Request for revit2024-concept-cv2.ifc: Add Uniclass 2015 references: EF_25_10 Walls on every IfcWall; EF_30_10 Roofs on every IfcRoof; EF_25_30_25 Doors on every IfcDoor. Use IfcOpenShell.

First a look at what the model holds.

```python
import ifcopenshell

model = ifcopenshell.open("revit2024-concept-cv2.ifc")
print(model.schema)
print("classifications:", [c.Name for c in model.by_type("IfcClassification")])
for ifc_class in ("IfcDoor", "IfcRoof", "IfcStair", "IfcWall", "IfcWindow"):
    print(ifc_class, len(model.by_type(ifc_class)))
```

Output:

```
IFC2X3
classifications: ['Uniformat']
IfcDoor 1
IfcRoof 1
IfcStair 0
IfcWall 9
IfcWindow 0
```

```python
import ifcopenshell
import ifcopenshell.api.classification

model = ifcopenshell.open("revit2024-concept-cv2.ifc")

# IFC2X3 requires Source and Edition and has no link from the project to the system.
system = model.create_entity("IfcClassification", Source="NBS", Edition="2015", Name="Uniclass 2015")

codes = {
    "IfcWall": ("EF_25_10", "Walls"),
    "IfcRoof": ("EF_30_10", "Roofs"),
    "IfcDoor": ("EF_25_30_25", "Doors"),
}
for ifc_class, (code, name) in codes.items():
    products = model.by_type(ifc_class)
    ifcopenshell.api.classification.add_reference(
        model, products=products, classification=system, identification=code, name=name
    )
    print(code, len(products))

model.write("revit2024-concept-cv2-out.ifc")
```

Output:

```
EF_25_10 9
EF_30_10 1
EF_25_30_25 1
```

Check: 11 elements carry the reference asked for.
